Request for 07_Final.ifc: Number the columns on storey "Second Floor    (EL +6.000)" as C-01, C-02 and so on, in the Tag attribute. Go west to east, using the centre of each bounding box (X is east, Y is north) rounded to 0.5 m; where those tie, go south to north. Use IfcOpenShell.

First a look at what the model holds.

```python
import ifcopenshell
import ifcopenshell.util.element
import ifcopenshell.util.placement

model = ifcopenshell.open("07_Final.ifc")
print(model.schema)
storey = next(s for s in model.by_type("IfcBuildingStorey") if s.Name == "Second Floor    (EL +6.000)")
columns = [e for e in ifcopenshell.util.element.get_decomposition(storey) if e.is_a("IfcColumn")]
for e in sorted(columns, key=lambda e: e.id()):
    origin = ifcopenshell.util.placement.get_local_placement(e.ObjectPlacement)[:3, 3]
    print(e.id(), e.Tag, e.Name, origin.round(2) + 0.0, sep=" | ")
```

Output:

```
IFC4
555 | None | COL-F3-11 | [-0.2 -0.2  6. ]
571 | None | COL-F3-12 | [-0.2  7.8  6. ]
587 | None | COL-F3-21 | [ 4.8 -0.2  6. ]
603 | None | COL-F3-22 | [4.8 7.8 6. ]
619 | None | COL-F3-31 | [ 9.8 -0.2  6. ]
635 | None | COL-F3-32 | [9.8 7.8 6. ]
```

```python
import ifcopenshell
import ifcopenshell.geom
import ifcopenshell.util.element
import ifcopenshell.util.shape

model = ifcopenshell.open("07_Final.ifc")
settings = ifcopenshell.geom.settings()
settings.set("use-world-coords", True)


def centre(element):
    shape = ifcopenshell.geom.create_shape(settings, element)
    return ifcopenshell.util.shape.get_bbox_centroid(shape.geometry)


storey = next(s for s in model.by_type("IfcBuildingStorey") if s.Name == "Second Floor    (EL +6.000)")
columns = [e for e in ifcopenshell.util.element.get_decomposition(storey) if e.is_a("IfcColumn")]

# Insertion points can sit at a corner or the storey origin, so sort by the geometry (in metres).
centres = {e: centre(e) for e in columns}
columns.sort(key=lambda e: (round(centres[e][0] / 0.5), centres[e][1]))

for i, e in enumerate(columns, start=1):
    number = f"C-{i:02d}"
    e.Tag = number
    print(e.id(), number)

model.write("07_Final_updated.ifc")
```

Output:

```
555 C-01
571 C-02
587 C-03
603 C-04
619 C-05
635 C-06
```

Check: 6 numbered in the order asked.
